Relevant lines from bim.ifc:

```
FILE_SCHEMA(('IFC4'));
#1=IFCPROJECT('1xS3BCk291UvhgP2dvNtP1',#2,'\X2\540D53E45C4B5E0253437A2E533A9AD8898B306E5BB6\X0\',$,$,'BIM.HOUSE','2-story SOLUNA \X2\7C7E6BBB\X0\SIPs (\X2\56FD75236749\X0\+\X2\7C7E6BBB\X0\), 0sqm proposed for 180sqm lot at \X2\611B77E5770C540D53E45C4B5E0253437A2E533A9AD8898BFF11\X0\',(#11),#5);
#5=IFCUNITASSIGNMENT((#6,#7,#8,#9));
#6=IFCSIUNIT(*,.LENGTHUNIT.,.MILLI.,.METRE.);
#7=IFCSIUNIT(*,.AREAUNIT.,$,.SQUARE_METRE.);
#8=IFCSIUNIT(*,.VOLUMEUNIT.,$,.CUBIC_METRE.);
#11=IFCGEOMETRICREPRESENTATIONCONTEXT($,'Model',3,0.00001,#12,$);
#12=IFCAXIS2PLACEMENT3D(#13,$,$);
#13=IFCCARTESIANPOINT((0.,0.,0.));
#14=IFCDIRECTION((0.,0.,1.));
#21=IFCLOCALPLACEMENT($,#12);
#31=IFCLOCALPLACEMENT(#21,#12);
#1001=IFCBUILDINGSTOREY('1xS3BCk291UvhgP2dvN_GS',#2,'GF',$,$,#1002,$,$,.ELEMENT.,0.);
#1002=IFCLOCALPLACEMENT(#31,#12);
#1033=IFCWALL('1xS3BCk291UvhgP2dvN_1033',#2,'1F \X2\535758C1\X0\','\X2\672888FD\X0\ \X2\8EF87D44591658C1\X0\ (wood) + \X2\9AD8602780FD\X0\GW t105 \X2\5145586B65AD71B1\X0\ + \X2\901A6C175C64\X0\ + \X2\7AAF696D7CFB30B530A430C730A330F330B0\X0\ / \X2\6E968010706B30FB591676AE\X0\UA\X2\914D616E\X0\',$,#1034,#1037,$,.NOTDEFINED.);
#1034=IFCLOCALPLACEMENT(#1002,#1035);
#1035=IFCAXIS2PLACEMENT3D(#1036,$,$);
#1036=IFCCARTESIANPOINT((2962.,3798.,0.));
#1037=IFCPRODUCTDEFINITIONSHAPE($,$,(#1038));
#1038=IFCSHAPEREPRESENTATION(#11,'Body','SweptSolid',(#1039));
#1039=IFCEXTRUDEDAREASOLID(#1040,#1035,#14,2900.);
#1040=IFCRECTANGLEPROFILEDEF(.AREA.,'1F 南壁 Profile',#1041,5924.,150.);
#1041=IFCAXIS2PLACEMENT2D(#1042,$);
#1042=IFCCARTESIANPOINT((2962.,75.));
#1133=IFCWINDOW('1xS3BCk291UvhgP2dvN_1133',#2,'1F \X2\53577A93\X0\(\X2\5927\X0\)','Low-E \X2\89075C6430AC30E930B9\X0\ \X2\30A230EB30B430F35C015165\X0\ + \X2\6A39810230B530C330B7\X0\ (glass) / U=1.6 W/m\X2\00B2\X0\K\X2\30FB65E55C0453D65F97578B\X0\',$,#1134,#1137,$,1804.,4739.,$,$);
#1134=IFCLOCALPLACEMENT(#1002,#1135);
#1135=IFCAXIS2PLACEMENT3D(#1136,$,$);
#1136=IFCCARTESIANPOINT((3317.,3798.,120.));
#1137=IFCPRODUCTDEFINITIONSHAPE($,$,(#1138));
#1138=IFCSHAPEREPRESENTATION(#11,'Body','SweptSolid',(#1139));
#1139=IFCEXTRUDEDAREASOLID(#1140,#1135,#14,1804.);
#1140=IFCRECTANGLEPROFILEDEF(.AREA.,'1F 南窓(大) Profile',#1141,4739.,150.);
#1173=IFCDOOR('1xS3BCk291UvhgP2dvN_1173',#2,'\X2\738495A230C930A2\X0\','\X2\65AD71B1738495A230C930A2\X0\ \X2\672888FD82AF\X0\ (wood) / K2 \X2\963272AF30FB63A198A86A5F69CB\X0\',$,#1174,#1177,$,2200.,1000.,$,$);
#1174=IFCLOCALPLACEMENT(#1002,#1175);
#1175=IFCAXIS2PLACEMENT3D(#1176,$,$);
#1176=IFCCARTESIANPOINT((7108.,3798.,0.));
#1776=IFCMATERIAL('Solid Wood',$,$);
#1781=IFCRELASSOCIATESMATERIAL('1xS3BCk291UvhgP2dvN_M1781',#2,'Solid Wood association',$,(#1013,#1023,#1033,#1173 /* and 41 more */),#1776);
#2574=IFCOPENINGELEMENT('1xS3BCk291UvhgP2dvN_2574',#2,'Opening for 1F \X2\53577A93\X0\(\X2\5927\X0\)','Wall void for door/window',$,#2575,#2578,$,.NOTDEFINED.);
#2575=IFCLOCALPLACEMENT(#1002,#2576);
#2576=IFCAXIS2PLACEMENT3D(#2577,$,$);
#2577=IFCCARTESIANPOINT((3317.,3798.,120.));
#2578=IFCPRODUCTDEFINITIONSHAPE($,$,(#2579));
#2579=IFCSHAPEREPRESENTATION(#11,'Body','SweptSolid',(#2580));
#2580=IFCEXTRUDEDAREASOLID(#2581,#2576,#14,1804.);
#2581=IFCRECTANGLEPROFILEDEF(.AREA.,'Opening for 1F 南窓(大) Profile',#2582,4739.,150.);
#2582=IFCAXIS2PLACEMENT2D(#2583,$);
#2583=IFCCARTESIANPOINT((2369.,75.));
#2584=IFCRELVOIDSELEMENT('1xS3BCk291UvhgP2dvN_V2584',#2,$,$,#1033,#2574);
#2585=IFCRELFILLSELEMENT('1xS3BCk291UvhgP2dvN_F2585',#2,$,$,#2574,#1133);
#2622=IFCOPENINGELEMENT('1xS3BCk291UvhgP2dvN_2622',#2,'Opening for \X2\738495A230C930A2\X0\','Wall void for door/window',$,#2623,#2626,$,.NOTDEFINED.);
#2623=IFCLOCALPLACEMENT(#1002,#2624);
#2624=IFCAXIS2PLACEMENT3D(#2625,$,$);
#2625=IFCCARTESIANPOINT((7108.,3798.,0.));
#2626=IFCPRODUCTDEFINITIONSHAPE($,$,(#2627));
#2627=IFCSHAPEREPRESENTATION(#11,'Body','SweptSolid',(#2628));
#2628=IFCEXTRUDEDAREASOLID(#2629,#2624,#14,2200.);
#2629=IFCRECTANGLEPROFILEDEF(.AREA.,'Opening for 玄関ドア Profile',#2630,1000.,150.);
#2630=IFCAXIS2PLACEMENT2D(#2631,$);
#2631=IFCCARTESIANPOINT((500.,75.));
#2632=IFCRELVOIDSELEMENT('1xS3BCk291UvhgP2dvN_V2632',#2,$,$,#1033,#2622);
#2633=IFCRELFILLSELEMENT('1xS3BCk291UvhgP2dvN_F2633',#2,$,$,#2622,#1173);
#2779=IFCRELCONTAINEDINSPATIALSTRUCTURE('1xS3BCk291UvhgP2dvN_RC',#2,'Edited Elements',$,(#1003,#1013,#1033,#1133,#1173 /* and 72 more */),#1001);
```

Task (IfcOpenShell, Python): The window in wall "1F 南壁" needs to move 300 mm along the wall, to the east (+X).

```python
import ifcopenshell
import ifcopenshell.api.geometry
import ifcopenshell.util.placement
import ifcopenshell.util.unit

model = ifcopenshell.open("bim.ifc")
unit_scale = ifcopenshell.util.unit.calculate_unit_scale(model)

window = model.by_guid("1xS3BCk291UvhgP2dvN_1133")
opening = window.FillsVoids[0].RelatingOpeningElement
wall = opening.VoidsElements[0].RelatingBuildingElement

wall_matrix = ifcopenshell.util.placement.get_local_placement(wall.ObjectPlacement)
shift = wall_matrix[:3, 0] * 0.3 / unit_scale
before = ifcopenshell.util.placement.get_local_placement(window.ObjectPlacement)[:3, 3].copy()

# The window is not placed relative to its opening, so move both.
for product in (opening, window):
    matrix = ifcopenshell.util.placement.get_local_placement(product.ObjectPlacement)
    matrix[:3, 3] += shift
    ifcopenshell.api.geometry.edit_object_placement(model, product=product, matrix=matrix, is_si=False)

after = ifcopenshell.util.placement.get_local_placement(window.ObjectPlacement)[:3, 3]
print("window moved by", (after - before).round(3) + 0.0)

model.write("bim_rev.ifc")
```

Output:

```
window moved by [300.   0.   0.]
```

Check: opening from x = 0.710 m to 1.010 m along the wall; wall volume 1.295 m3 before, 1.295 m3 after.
